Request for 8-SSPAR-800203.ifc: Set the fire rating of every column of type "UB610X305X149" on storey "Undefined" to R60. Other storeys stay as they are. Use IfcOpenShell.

First a look at what the model holds.

```python
import ifcopenshell
import ifcopenshell.util.element

model = ifcopenshell.open("8-SSPAR-800203.ifc")
print(model.schema)
storey = next(s for s in model.by_type("IfcBuildingStorey") if s.Name == "Undefined")
columns = [e for e in ifcopenshell.util.element.get_decomposition(storey) if e.is_a("IfcColumn")]
seen = {}
for e in columns:
    element_type = ifcopenshell.util.element.get_type(e)
    key = (element_type.Name if element_type != e and element_type else None, ifcopenshell.util.element.get_pset(e, "Pset_ColumnCommon", "FireRating"))
    seen[key] = seen.get(key, 0) + 1
for (name, value), count in sorted(seen.items(), key=str):
    print(count, "x", name, "|", value)
```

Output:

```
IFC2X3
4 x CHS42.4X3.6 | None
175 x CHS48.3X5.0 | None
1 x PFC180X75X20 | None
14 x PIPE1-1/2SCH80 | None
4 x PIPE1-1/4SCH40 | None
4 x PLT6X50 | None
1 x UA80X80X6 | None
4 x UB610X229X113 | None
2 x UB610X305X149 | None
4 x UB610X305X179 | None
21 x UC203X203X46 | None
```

```python
import ifcopenshell
import ifcopenshell.api.pset
import ifcopenshell.util.element

model = ifcopenshell.open("8-SSPAR-800203.ifc")

storey = next(s for s in model.by_type("IfcBuildingStorey") if s.Name == "Undefined")
columns = [e for e in ifcopenshell.util.element.get_decomposition(storey) if e.is_a("IfcColumn")]

count = 0
for e in columns:
    element_type = ifcopenshell.util.element.get_type(e)
    if element_type in (None, e) or element_type.Name != "UB610X305X149":
        continue
    # add_pset returns the element's existing set when there is one.
    pset = ifcopenshell.api.pset.add_pset(model, product=e, name="Pset_ColumnCommon")
    ifcopenshell.api.pset.edit_pset(model, pset=pset, properties={"FireRating": "R60"})
    count += 1

print(count, "columns updated")

model.write("8-SSPAR-800203_rev.ifc")
```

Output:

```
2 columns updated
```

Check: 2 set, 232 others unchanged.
